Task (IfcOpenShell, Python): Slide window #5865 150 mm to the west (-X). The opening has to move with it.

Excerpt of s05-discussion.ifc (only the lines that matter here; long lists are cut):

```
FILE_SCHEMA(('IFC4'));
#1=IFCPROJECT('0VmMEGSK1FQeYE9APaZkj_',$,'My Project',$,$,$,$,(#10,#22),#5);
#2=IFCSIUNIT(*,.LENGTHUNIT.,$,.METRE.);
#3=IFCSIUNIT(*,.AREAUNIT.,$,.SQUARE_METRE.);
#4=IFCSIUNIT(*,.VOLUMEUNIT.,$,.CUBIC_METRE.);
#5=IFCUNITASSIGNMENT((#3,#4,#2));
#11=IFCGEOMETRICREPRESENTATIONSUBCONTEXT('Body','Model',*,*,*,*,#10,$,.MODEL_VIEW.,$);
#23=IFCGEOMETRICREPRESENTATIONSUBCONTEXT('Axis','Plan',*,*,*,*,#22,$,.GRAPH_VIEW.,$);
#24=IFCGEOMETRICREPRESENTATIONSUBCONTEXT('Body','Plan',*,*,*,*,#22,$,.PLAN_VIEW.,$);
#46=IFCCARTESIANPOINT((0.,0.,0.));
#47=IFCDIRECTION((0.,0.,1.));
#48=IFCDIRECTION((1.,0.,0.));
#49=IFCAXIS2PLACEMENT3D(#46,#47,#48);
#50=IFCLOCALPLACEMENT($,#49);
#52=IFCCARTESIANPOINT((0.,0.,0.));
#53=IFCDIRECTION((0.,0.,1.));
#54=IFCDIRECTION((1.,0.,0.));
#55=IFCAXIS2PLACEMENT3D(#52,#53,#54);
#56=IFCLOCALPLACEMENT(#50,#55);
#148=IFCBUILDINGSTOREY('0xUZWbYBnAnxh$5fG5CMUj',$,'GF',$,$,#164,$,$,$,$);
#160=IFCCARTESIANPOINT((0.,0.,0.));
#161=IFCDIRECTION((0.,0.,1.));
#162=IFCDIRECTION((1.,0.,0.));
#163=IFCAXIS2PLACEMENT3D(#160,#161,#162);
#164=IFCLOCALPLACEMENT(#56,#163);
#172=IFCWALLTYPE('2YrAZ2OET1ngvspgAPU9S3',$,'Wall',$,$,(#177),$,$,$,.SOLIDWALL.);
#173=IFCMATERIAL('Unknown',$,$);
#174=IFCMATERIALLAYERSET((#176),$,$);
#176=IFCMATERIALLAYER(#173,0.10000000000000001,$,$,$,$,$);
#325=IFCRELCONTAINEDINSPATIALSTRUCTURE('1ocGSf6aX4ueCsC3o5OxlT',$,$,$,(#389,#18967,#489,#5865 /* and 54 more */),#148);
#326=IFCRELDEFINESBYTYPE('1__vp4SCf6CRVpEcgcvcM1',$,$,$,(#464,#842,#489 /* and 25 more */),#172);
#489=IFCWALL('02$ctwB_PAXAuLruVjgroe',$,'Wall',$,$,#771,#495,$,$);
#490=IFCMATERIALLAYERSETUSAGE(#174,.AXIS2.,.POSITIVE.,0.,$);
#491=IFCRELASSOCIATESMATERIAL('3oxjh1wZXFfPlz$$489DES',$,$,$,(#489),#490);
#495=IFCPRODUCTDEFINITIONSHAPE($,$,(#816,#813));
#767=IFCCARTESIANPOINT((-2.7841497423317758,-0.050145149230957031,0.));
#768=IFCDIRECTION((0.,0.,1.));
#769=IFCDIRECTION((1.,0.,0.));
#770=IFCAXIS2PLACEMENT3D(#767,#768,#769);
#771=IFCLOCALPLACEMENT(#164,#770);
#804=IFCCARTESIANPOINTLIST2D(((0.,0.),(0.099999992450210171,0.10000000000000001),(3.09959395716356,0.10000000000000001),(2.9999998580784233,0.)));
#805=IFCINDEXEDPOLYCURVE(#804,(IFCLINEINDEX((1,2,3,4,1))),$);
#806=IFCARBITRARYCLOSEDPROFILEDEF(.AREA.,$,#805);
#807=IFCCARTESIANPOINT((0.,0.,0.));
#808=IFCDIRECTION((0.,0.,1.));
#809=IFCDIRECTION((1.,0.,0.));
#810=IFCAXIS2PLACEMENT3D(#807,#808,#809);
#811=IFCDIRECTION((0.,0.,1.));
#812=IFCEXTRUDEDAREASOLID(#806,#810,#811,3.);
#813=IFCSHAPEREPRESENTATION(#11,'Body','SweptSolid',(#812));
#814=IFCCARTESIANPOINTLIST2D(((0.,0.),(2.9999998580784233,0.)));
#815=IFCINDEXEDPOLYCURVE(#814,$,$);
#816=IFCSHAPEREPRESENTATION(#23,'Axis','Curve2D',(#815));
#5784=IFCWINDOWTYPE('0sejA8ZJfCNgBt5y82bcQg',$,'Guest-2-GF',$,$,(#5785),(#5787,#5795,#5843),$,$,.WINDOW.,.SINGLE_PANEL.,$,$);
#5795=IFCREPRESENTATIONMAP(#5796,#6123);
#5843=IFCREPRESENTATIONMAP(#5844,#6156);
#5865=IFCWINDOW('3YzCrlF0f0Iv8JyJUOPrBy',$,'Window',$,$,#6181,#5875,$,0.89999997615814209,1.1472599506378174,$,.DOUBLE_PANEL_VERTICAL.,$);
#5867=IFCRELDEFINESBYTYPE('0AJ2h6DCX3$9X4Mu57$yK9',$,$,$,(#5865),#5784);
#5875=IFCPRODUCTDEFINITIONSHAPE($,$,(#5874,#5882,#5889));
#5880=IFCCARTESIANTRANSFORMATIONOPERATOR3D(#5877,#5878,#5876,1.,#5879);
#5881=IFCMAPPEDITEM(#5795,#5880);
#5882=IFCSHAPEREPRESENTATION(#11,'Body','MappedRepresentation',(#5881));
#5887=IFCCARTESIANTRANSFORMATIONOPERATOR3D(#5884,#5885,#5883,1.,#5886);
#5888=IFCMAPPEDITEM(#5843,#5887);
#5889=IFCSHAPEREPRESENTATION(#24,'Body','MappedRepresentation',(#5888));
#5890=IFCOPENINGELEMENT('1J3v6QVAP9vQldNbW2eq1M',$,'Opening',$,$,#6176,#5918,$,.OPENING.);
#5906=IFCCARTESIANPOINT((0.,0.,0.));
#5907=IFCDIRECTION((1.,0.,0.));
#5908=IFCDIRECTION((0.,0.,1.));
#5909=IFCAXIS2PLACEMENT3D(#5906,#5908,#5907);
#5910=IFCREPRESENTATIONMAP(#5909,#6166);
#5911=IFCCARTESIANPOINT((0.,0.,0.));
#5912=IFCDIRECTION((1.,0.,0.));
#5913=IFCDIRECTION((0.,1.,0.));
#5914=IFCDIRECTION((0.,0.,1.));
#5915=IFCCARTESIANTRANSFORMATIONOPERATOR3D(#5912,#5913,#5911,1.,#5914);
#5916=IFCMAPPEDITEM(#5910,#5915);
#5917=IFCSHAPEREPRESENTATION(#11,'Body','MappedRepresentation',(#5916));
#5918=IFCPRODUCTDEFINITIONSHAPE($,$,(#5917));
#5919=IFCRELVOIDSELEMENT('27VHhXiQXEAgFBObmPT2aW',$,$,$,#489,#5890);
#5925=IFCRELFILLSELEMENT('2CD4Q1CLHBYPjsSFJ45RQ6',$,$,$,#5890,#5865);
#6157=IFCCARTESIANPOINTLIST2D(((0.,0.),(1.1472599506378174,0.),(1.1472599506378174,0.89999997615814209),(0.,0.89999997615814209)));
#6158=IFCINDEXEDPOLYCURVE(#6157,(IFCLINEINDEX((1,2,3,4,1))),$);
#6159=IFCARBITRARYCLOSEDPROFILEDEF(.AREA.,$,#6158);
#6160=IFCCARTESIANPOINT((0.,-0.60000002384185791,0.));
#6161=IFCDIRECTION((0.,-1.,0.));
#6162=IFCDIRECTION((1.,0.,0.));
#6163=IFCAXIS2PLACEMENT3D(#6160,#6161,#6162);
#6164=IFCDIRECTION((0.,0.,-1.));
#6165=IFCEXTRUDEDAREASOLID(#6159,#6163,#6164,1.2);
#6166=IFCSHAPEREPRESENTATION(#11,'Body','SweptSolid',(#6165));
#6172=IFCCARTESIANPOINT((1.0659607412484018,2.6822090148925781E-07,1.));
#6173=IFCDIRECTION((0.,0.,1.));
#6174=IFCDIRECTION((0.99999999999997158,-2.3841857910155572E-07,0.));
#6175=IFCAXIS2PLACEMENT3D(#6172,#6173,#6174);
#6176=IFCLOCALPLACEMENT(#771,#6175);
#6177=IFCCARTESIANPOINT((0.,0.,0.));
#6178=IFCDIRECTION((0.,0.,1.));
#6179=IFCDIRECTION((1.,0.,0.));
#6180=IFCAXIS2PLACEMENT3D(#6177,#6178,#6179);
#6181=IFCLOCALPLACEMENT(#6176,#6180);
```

```python
import ifcopenshell
import ifcopenshell.api.geometry
import ifcopenshell.util.placement

model = ifcopenshell.open("s05-discussion.ifc")

window = model.by_guid("3YzCrlF0f0Iv8JyJUOPrBy")
opening = window.FillsVoids[0].RelatingOpeningElement
wall = opening.VoidsElements[0].RelatingBuildingElement

wall_matrix = ifcopenshell.util.placement.get_local_placement(wall.ObjectPlacement)
shift = wall_matrix[:3, 0] * -0.15
before = ifcopenshell.util.placement.get_local_placement(window.ObjectPlacement)[:3, 3].copy()

# The window is placed relative to its opening, so it follows when the opening moves.
matrix = ifcopenshell.util.placement.get_local_placement(opening.ObjectPlacement)
matrix[:3, 3] += shift
ifcopenshell.api.geometry.edit_object_placement(
    model, product=opening, matrix=matrix, is_si=False, should_transform_children=True
)

after = ifcopenshell.util.placement.get_local_placement(window.ObjectPlacement)[:3, 3]
print("window moved by", (after - before).round(3) + 0.0)

model.write("s05-discussion_rev.ifc")
```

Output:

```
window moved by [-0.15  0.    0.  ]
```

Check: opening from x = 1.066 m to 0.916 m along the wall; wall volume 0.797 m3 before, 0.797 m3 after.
